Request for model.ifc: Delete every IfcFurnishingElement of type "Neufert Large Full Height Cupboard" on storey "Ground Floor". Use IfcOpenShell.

First a look at what the model holds.

```python
import ifcopenshell
import ifcopenshell.util.element

model = ifcopenshell.open("model.ifc")
print(model.schema)
storey = next(s for s in model.by_type("IfcBuildingStorey") if s.Name == "Ground Floor")
furniture = [e for e in ifcopenshell.util.element.get_decomposition(storey) if e.is_a("IfcFurnishingElement")]
seen = {}
for e in furniture:
    element_type = ifcopenshell.util.element.get_type(e)
    name = element_type.Name if element_type not in (None, e) else None
    seen[name] = seen.get(name, 0) + 1
for name, count in sorted(seen.items(), key=str):
    print(count, "x", name)
```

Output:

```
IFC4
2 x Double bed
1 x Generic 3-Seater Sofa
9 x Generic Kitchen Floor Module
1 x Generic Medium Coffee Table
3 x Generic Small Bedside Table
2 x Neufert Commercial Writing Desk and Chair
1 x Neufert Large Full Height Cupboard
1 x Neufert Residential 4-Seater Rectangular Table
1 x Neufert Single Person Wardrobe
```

```python
import ifcopenshell
import ifcopenshell.api.root
import ifcopenshell.util.element

model = ifcopenshell.open("model.ifc")

storey = next(s for s in model.by_type("IfcBuildingStorey") if s.Name == "Ground Floor")
furniture = [e for e in ifcopenshell.util.element.get_decomposition(storey) if e.is_a("IfcFurnishingElement")]
targets = [e for e in furniture if (t := ifcopenshell.util.element.get_type(e)) not in (None, e) and t.Name == "Neufert Large Full Height Cupboard"]

for e in targets:
    ifcopenshell.api.root.remove_product(model, product=e)
print(len(targets), "removed")

model.write("model_rev.ifc")
```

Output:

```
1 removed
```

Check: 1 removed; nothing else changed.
